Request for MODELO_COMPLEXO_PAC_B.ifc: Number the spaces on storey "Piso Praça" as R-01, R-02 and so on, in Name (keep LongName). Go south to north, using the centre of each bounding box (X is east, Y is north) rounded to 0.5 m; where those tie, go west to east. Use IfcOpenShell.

First a look at what the model holds.

```python
import ifcopenshell
import ifcopenshell.util.element
import ifcopenshell.util.placement

model = ifcopenshell.open("MODELO_COMPLEXO_PAC_B.ifc")
print(model.schema)
storey = next(s for s in model.by_type("IfcBuildingStorey") if s.Name == "Piso Praça")
spaces = [e for e in ifcopenshell.util.element.get_decomposition(storey) if e.is_a("IfcSpace")]
for e in sorted(spaces, key=lambda e: e.id()):
    origin = ifcopenshell.util.placement.get_local_placement(e.ObjectPlacement)[:3, 3]
    print(e.id(), e.Name, e.LongName, origin.round(2) + 0.0, sep=" | ")
```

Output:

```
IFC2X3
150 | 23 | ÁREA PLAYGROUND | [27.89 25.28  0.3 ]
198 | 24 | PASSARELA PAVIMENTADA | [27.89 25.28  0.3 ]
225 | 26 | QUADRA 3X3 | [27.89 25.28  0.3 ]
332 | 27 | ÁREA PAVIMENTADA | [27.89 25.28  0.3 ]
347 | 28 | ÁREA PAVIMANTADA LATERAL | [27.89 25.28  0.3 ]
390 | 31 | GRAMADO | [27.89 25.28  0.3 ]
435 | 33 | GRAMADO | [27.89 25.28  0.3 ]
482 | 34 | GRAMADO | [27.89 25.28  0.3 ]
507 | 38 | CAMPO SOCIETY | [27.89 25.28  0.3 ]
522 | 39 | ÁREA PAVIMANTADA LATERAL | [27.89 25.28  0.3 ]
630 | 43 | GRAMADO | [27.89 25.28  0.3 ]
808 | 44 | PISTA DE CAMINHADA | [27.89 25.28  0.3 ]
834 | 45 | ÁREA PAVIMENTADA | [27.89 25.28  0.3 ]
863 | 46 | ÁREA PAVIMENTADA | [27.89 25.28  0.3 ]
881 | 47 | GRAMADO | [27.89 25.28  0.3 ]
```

```python
import ifcopenshell
import ifcopenshell.geom
import ifcopenshell.util.element
import ifcopenshell.util.shape

model = ifcopenshell.open("MODELO_COMPLEXO_PAC_B.ifc")
settings = ifcopenshell.geom.settings()
settings.set("use-world-coords", True)


def centre(element):
    shape = ifcopenshell.geom.create_shape(settings, element)
    return ifcopenshell.util.shape.get_bbox_centroid(shape.geometry)


storey = next(s for s in model.by_type("IfcBuildingStorey") if s.Name == "Piso Praça")
spaces = [e for e in ifcopenshell.util.element.get_decomposition(storey) if e.is_a("IfcSpace")]

# Insertion points can sit at a corner or the storey origin, so sort by the geometry (in metres).
centres = {e: centre(e) for e in spaces}
spaces.sort(key=lambda e: (round(centres[e][1] / 0.5), centres[e][0]))

for i, e in enumerate(spaces, start=1):
    number = f"R-{i:02d}"
    e.Name = number
    print(e.id(), number)

model.write("MODELO_COMPLEXO_PAC_B_edited.ifc")
```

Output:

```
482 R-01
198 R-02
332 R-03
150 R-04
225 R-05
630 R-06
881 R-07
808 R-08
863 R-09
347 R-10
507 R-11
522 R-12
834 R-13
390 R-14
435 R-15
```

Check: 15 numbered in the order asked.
